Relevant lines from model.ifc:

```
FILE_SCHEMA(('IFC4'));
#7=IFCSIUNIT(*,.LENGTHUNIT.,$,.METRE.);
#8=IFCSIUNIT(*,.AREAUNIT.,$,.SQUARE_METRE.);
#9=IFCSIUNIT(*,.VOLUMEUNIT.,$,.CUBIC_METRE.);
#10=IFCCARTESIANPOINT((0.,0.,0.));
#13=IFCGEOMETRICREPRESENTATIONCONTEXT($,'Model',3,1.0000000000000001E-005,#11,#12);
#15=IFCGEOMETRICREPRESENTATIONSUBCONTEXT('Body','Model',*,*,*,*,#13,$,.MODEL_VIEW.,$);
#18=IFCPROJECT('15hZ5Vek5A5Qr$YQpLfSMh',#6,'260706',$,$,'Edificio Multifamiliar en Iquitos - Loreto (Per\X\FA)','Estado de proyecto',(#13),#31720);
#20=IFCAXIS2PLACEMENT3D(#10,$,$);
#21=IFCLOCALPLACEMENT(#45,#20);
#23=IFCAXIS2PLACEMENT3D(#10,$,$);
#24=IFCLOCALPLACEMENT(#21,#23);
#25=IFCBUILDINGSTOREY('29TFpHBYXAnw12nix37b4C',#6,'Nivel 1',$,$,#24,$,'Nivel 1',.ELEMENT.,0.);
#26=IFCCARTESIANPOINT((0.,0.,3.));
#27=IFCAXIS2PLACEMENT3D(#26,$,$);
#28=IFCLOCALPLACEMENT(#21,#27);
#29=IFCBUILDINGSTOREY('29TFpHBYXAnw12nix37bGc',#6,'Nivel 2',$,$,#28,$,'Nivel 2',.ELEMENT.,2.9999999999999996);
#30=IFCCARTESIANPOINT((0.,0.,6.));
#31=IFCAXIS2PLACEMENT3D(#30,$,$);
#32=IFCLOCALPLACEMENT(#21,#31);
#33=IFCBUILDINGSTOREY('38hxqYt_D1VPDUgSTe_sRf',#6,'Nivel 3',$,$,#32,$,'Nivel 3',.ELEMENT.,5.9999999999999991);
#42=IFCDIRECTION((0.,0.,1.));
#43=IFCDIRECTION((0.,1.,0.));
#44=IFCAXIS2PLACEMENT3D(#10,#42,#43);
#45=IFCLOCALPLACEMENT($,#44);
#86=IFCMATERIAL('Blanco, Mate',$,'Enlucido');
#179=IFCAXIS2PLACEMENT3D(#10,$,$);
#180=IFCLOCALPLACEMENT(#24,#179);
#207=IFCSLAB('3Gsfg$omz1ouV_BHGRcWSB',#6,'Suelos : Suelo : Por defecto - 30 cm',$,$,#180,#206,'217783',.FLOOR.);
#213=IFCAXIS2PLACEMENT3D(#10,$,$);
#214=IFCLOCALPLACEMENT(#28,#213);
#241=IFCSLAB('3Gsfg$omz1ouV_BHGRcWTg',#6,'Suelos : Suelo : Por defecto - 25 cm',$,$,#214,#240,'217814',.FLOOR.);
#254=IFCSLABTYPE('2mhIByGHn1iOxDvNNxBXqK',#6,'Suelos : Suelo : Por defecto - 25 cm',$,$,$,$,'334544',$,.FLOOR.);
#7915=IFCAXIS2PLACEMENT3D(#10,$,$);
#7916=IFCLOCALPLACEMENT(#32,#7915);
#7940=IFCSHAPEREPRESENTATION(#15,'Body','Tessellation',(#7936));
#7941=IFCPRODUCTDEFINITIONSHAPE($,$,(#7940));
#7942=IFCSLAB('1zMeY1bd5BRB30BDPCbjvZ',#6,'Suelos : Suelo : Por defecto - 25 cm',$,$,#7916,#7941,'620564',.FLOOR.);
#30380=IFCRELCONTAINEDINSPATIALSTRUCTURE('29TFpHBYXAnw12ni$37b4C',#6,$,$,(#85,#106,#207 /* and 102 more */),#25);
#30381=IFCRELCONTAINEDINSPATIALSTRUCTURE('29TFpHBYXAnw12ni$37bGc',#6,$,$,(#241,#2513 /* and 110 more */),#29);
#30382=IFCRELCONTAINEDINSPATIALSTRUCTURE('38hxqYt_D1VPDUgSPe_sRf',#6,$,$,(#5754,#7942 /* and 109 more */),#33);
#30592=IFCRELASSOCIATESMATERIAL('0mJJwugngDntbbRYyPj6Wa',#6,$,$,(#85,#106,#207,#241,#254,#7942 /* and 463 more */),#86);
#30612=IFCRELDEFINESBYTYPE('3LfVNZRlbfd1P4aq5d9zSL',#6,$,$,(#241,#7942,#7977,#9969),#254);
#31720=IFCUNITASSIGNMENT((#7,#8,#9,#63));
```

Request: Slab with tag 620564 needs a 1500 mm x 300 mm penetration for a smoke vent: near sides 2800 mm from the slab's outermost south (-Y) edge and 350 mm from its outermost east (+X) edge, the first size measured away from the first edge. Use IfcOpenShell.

```python
import numpy as np
import ifcopenshell
import ifcopenshell.api.feature
import ifcopenshell.api.geometry
import ifcopenshell.api.root
import ifcopenshell.geom
import ifcopenshell.util.placement
import ifcopenshell.util.representation
import ifcopenshell.util.shape
import ifcopenshell.util.unit

model = ifcopenshell.open("model.ifc")
unit_scale = ifcopenshell.util.unit.calculate_unit_scale(model)
settings = ifcopenshell.geom.settings()


def volume(element):
    """Net volume in cubic metres, openings subtracted."""
    shape = ifcopenshell.geom.create_shape(settings, element)
    return ifcopenshell.util.shape.get_volume(shape.geometry)


slab = model.by_id(7942)
before = volume(slab)

# Extent in the slab's own axes, in metres. The edges named are its -X and -Y sides.
slab_shape = ifcopenshell.geom.create_shape(settings, slab)
vertices = ifcopenshell.util.shape.get_vertices(slab_shape.geometry)
x_min, y_min, bottom = vertices.min(axis=0)
top = vertices[:, 2].max()

opening = ifcopenshell.api.root.create_entity(model, ifc_class="IfcOpeningElement", name="Smoke vent opening", predefined_type="OPENING")
context = ifcopenshell.util.representation.get_context(model, "Model", "Body", "MODEL_VIEW")
width, depth = 1.5, 0.3
outline = [(0.0, 0.0), (width, 0.0), (width, depth), (0.0, depth), (0.0, 0.0)]
# Overshoot both faces by 50 mm so the cut is clean.
shape = ifcopenshell.api.geometry.add_slab_representation(
    model, context=context, depth=top - bottom + 0.1, polyline=outline
)
ifcopenshell.api.geometry.assign_representation(model, product=opening, representation=shape)

matrix = ifcopenshell.util.placement.get_local_placement(slab.ObjectPlacement)
matrix[:, 3] = matrix @ np.append(np.array([x_min + 2.8, y_min + 0.35, bottom - 0.05]) / unit_scale, 1.0)
ifcopenshell.api.geometry.edit_object_placement(model, product=opening, matrix=matrix, is_si=False)
ifcopenshell.api.feature.add_feature(model, feature=opening, element=slab)

after = volume(slab)

print(f"slab volume {before:.3f} -> {after:.3f} m3")

model.write("model_updated.ifc")
```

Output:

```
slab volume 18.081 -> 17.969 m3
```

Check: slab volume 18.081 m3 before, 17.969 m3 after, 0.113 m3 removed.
